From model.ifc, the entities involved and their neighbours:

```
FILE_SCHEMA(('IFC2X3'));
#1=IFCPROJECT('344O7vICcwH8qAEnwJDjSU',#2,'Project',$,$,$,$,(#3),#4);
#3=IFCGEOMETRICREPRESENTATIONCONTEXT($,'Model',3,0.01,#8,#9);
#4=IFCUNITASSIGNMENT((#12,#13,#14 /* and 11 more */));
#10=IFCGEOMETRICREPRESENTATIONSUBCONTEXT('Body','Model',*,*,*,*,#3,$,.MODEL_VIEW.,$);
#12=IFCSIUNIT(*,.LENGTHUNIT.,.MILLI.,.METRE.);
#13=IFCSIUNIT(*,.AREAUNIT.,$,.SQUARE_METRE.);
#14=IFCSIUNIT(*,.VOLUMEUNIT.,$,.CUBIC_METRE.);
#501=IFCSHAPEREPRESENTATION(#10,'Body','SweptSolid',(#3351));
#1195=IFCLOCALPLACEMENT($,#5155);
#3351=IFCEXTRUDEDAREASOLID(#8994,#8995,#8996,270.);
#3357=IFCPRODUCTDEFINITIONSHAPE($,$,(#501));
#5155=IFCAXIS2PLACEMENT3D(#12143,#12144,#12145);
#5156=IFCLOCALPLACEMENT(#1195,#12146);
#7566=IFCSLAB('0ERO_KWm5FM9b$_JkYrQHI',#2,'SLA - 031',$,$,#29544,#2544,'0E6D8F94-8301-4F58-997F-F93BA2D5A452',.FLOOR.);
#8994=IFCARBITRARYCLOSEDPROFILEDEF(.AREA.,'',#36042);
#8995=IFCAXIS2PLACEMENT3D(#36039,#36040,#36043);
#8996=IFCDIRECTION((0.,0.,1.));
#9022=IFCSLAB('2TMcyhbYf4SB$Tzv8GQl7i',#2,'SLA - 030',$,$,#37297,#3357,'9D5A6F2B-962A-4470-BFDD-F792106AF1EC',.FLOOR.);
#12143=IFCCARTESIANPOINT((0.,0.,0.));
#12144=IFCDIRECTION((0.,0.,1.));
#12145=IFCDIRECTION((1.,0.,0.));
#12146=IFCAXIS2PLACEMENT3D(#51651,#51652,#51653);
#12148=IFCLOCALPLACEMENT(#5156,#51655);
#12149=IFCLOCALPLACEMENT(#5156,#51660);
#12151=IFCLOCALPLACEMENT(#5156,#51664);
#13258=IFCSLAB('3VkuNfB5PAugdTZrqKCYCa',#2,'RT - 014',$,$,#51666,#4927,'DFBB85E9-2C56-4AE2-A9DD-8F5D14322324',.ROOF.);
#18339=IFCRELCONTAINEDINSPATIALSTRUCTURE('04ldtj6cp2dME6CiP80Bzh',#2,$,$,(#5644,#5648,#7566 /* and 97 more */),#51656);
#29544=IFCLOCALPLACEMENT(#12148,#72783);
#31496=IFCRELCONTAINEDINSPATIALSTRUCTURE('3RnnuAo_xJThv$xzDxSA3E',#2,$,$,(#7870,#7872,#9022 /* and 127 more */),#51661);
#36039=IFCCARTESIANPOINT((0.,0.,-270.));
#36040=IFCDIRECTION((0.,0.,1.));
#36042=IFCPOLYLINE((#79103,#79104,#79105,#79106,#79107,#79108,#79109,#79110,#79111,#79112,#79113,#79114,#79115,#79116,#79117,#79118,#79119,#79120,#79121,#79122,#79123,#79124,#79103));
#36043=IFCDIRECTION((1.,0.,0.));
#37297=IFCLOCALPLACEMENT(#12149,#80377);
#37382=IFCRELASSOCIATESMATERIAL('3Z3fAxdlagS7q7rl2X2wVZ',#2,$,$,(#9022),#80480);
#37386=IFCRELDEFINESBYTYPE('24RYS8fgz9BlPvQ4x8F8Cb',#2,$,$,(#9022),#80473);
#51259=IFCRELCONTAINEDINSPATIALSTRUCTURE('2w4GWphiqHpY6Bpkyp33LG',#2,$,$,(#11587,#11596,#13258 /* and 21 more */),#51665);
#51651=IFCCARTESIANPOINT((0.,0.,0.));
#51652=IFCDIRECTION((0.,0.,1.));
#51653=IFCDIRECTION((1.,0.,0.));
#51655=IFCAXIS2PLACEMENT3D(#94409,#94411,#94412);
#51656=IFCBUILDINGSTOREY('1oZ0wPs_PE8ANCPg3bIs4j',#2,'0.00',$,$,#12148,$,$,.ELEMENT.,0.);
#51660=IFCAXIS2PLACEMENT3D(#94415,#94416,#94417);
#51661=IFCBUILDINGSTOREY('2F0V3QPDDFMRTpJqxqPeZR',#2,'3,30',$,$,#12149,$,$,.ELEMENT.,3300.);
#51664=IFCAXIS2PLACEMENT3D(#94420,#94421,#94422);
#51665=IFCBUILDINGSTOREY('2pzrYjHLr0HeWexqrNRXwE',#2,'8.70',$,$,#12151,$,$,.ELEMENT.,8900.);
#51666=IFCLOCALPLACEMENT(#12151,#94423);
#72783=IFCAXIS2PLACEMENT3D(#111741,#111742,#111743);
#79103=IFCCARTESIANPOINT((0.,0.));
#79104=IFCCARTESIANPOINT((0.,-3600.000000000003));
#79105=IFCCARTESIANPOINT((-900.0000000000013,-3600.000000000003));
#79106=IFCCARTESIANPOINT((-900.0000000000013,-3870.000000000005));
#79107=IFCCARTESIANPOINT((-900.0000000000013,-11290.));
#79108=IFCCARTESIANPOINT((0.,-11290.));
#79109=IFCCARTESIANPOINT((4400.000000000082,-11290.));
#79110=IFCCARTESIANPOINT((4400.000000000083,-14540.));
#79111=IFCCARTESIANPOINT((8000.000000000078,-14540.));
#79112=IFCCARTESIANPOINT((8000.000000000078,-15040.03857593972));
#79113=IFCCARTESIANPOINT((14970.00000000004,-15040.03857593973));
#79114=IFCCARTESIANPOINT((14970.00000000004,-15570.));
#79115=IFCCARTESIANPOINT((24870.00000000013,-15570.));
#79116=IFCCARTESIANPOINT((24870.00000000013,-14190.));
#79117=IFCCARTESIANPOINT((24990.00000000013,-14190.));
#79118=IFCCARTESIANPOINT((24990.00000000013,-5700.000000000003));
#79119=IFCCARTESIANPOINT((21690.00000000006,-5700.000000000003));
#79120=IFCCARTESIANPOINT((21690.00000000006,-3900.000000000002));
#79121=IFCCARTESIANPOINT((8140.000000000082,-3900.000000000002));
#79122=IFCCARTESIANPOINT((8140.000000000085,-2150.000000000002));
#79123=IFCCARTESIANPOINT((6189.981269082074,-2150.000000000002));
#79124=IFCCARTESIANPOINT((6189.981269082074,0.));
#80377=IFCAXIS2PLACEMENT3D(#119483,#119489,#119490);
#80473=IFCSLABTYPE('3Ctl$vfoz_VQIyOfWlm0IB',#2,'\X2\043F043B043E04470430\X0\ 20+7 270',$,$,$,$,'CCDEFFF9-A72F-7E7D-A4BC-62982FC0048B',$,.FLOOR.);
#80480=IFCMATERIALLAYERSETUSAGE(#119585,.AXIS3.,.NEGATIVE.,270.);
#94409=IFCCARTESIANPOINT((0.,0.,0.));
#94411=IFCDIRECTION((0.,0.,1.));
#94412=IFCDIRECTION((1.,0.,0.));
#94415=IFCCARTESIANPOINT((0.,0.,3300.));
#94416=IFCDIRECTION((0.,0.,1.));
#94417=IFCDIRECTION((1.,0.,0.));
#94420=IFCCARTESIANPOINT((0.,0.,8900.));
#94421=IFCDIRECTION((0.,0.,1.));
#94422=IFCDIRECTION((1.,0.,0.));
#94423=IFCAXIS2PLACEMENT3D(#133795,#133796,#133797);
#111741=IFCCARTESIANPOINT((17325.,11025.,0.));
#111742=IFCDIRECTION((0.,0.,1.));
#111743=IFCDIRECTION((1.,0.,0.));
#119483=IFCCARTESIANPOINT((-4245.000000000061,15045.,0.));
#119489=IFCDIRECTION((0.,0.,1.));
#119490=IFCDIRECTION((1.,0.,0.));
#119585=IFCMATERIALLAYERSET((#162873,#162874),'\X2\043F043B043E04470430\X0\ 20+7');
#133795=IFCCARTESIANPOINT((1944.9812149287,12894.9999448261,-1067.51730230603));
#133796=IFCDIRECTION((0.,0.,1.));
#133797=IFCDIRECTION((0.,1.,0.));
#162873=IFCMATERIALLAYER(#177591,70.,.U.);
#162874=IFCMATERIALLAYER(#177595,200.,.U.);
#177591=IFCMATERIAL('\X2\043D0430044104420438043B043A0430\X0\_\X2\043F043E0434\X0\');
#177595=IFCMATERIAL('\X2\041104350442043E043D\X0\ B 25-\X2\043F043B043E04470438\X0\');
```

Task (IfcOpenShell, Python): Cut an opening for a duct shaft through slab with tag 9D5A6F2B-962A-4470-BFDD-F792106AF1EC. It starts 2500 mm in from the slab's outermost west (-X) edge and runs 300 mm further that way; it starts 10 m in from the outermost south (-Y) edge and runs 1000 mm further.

```python
import numpy as np
import ifcopenshell
import ifcopenshell.api.feature
import ifcopenshell.api.geometry
import ifcopenshell.api.root
import ifcopenshell.geom
import ifcopenshell.util.placement
import ifcopenshell.util.representation
import ifcopenshell.util.shape
import ifcopenshell.util.unit

model = ifcopenshell.open("model.ifc")
unit_scale = ifcopenshell.util.unit.calculate_unit_scale(model)
settings = ifcopenshell.geom.settings()


def volume(element):
    """Net volume in cubic metres, openings subtracted."""
    shape = ifcopenshell.geom.create_shape(settings, element)
    return ifcopenshell.util.shape.get_volume(shape.geometry)


slab = model.by_guid("2TMcyhbYf4SB$Tzv8GQl7i")
before = volume(slab)

# Extent in the slab's own axes, in metres. The edges named are its -X and -Y sides.
slab_shape = ifcopenshell.geom.create_shape(settings, slab)
vertices = ifcopenshell.util.shape.get_vertices(slab_shape.geometry)
x_min, y_min, bottom = vertices.min(axis=0)
top = vertices[:, 2].max()

opening = ifcopenshell.api.root.create_entity(model, ifc_class="IfcOpeningElement", name="Duct shaft opening")
context = ifcopenshell.util.representation.get_context(model, "Model", "Body", "MODEL_VIEW")
width, depth = 0.3, 1
outline = [(0.0, 0.0), (width, 0.0), (width, depth), (0.0, depth), (0.0, 0.0)]
# Overshoot both faces by 50 mm so the cut is clean.
shape = ifcopenshell.api.geometry.add_slab_representation(
    model, context=context, depth=top - bottom + 0.1, polyline=outline
)
ifcopenshell.api.geometry.assign_representation(model, product=opening, representation=shape)

matrix = ifcopenshell.util.placement.get_local_placement(slab.ObjectPlacement)
matrix[:, 3] = matrix @ np.append(np.array([x_min + 2.5, y_min + 10, bottom - 0.05]) / unit_scale, 1.0)
ifcopenshell.api.geometry.edit_object_placement(model, product=opening, matrix=matrix, is_si=False)
ifcopenshell.api.feature.add_feature(model, feature=opening, element=slab)

after = volume(slab)

print(f"slab volume {before:.3f} -> {after:.3f} m3")

model.write("model_updated.ifc")
```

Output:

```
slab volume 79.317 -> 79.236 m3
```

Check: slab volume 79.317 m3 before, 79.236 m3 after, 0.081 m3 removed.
